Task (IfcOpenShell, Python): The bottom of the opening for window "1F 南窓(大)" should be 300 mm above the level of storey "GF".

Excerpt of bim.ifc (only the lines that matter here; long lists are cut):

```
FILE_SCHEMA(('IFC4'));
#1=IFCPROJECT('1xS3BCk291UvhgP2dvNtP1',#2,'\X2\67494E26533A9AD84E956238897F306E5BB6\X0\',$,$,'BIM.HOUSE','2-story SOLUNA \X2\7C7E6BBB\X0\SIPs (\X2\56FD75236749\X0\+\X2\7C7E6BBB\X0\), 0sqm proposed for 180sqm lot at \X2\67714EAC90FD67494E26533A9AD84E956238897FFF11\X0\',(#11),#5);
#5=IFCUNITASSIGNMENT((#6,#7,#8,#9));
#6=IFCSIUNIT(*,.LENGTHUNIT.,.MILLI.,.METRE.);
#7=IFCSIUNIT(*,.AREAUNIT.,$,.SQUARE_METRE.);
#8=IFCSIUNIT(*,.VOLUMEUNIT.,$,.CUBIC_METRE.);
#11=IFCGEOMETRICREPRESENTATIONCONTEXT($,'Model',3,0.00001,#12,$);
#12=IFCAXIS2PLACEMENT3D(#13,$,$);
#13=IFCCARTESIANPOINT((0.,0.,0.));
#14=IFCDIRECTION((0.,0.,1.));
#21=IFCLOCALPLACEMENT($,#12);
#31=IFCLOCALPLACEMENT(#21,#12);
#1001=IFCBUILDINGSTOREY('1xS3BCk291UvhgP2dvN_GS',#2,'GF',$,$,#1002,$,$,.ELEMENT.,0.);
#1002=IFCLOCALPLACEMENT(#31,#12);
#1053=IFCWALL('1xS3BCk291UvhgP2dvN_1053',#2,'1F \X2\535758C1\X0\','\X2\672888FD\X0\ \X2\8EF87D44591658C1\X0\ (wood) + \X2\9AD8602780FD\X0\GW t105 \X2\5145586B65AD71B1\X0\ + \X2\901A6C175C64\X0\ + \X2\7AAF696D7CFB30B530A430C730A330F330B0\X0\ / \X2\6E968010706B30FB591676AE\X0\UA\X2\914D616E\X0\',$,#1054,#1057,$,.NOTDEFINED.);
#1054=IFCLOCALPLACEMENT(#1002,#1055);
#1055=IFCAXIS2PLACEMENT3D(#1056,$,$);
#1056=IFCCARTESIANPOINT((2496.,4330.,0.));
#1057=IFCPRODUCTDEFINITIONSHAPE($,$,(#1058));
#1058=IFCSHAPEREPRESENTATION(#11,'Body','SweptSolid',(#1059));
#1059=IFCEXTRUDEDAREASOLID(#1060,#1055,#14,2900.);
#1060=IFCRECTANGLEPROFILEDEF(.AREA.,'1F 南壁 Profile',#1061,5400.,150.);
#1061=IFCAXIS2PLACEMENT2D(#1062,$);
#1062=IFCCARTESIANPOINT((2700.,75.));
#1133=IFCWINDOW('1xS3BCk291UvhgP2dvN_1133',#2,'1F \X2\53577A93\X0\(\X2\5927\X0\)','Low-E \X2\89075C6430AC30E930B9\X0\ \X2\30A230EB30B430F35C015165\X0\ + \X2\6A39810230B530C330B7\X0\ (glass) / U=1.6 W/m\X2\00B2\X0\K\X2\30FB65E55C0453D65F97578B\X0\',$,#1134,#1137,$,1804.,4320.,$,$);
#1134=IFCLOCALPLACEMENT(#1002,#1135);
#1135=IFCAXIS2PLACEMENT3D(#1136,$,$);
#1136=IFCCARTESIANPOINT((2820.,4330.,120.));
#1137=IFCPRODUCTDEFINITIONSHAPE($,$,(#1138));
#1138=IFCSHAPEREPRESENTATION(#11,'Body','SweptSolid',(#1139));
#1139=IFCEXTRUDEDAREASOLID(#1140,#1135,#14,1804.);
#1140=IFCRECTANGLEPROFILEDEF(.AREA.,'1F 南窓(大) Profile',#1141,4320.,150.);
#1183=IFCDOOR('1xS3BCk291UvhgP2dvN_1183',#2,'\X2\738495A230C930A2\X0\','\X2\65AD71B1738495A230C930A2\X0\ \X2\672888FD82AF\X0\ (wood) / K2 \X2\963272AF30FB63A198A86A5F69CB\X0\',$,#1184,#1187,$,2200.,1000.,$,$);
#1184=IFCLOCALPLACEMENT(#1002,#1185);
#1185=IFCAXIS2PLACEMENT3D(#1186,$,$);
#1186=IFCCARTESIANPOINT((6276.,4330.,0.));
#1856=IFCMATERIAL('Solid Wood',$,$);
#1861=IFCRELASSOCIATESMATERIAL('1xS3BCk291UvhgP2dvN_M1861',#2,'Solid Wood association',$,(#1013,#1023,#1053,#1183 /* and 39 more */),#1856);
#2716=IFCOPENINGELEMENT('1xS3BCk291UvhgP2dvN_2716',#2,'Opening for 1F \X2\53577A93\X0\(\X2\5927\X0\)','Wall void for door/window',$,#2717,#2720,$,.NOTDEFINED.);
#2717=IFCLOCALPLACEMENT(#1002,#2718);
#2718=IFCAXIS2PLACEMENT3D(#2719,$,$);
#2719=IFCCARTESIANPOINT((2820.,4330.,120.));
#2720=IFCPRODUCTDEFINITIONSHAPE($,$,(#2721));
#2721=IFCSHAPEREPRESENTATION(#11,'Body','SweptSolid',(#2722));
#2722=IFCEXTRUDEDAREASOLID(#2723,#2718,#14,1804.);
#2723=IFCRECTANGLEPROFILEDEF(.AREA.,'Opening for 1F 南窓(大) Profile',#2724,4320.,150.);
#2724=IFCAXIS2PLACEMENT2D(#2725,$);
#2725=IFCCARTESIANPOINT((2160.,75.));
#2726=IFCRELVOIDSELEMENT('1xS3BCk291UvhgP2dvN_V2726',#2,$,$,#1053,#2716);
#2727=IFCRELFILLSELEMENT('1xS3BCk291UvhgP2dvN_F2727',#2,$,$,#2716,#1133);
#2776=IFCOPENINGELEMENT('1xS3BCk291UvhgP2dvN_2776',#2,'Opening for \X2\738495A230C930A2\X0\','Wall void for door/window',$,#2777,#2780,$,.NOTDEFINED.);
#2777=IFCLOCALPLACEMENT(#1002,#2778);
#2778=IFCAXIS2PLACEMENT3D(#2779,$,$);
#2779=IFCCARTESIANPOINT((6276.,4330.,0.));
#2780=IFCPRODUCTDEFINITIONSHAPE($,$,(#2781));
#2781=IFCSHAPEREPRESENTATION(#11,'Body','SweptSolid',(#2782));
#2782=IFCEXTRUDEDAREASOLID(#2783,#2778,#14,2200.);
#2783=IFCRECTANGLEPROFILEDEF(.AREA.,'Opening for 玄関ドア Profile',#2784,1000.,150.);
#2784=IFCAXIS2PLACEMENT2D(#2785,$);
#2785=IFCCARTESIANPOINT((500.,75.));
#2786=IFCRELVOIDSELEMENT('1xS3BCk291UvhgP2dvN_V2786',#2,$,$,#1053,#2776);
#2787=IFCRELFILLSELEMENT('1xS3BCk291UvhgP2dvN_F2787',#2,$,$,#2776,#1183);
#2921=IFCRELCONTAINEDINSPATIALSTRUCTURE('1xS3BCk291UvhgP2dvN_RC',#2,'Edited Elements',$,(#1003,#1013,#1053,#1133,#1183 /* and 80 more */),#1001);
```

```python
import numpy as np
import ifcopenshell
import ifcopenshell.api.geometry
import ifcopenshell.geom
import ifcopenshell.util.element
import ifcopenshell.util.placement
import ifcopenshell.util.shape
import ifcopenshell.util.unit

model = ifcopenshell.open("bim.ifc")
unit_scale = ifcopenshell.util.unit.calculate_unit_scale(model)

window = model.by_id(1133)
opening = window.FillsVoids[0].RelatingOpeningElement
storey = ifcopenshell.util.element.get_container(window, ifc_class="IfcBuildingStorey")
level = ifcopenshell.util.placement.get_local_placement(storey.ObjectPlacement)[2, 3]

# The opening's origin need not be at the sill, so measure its lowest point.
shape = ifcopenshell.geom.create_shape(ifcopenshell.geom.settings(), opening)
bottom = ifcopenshell.util.shape.get_shape_bottom_elevation(shape, shape.geometry) / unit_scale
dz = level + 0.3 / unit_scale - bottom

shift = np.array([0.0, 0.0, dz])
# The window is not placed relative to its opening, so move both.
for product in (opening, window):
    matrix = ifcopenshell.util.placement.get_local_placement(product.ObjectPlacement)
    matrix[:3, 3] += shift
    ifcopenshell.api.geometry.edit_object_placement(model, product=product, matrix=matrix, is_si=False)

print(f"moved by {dz * unit_scale:+.3f} m")

model.write("bim_updated.ifc")
```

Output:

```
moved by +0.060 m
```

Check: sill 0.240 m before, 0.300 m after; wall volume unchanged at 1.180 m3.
